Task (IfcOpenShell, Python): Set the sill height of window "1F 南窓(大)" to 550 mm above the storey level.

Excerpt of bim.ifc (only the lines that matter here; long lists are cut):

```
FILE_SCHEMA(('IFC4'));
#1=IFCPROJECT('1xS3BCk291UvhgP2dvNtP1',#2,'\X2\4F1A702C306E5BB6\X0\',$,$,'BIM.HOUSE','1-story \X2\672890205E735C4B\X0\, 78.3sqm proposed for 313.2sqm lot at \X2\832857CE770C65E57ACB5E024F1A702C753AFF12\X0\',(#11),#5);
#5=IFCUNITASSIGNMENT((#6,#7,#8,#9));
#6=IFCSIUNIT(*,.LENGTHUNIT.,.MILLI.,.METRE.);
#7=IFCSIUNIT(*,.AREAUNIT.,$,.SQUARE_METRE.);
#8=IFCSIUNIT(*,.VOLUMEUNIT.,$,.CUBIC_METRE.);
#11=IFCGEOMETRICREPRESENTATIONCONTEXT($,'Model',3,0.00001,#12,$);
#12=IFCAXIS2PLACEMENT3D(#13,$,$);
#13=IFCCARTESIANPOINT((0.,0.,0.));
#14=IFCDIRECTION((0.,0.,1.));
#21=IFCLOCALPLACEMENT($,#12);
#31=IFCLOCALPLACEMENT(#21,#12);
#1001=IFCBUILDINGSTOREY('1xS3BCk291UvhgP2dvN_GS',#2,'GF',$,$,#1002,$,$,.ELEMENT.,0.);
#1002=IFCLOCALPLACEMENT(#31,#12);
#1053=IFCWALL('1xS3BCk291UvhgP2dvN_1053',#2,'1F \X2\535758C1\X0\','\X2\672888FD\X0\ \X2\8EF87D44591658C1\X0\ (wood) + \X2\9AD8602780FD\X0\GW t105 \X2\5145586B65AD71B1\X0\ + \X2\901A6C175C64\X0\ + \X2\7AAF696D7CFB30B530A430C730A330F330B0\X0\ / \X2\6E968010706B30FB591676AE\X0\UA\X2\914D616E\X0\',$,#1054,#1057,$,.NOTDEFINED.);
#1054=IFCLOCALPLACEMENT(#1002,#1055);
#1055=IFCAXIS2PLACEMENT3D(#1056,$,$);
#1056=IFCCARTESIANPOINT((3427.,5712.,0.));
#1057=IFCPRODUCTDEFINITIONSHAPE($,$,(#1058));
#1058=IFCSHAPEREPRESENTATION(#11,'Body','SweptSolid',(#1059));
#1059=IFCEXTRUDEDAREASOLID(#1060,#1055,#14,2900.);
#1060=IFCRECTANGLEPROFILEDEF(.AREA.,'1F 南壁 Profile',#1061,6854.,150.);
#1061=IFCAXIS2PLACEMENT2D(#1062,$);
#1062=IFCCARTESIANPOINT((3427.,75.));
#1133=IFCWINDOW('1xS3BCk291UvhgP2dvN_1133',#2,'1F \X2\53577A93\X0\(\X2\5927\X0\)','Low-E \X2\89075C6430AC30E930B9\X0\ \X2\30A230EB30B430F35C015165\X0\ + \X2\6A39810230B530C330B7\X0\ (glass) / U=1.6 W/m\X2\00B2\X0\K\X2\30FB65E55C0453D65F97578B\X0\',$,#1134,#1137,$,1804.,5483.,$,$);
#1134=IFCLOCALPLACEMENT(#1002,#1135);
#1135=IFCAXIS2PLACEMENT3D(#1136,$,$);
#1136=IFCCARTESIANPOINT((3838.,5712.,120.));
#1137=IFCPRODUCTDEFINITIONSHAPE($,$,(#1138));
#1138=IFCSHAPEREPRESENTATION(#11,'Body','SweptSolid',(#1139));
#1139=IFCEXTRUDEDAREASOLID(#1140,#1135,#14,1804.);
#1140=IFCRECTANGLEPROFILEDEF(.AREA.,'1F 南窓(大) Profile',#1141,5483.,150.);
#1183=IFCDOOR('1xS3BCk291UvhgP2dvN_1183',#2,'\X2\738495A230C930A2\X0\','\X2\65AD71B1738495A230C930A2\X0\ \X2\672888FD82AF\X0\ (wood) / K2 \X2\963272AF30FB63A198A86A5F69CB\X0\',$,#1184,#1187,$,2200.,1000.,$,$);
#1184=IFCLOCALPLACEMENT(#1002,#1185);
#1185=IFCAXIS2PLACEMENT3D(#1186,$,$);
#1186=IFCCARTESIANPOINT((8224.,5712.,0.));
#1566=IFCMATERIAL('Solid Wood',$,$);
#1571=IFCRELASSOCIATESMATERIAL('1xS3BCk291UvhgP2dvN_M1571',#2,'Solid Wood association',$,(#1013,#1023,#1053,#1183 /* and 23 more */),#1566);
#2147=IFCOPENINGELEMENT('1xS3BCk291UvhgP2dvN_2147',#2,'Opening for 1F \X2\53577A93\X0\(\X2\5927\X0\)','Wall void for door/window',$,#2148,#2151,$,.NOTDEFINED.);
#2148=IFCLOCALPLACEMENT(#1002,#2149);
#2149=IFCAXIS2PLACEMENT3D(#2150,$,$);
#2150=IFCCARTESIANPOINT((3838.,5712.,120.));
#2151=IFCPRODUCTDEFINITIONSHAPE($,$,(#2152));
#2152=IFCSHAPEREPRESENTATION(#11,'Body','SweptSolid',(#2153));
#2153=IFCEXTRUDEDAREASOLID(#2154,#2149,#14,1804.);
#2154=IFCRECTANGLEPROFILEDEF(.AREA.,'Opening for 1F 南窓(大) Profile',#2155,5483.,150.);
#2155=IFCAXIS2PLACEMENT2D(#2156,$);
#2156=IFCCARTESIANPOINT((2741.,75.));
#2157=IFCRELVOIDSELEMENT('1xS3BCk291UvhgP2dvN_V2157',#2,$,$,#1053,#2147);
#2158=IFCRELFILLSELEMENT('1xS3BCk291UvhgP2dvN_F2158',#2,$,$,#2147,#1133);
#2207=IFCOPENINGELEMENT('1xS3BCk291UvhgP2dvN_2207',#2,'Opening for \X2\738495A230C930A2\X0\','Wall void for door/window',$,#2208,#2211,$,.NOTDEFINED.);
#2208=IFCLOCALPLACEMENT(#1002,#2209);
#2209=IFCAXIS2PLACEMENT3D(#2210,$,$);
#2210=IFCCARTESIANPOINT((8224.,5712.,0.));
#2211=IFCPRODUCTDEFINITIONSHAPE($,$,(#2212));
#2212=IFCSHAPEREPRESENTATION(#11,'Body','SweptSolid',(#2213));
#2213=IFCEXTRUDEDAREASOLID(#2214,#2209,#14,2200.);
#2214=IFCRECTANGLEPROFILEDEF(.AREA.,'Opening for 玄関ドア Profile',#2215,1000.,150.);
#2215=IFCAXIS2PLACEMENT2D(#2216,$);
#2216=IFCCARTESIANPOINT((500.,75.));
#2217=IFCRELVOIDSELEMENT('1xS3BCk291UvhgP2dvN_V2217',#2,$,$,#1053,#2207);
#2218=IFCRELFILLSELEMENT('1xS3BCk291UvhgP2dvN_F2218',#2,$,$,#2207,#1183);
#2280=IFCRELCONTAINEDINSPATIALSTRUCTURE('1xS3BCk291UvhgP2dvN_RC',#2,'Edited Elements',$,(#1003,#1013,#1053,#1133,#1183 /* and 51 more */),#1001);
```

```python
import numpy as np
import ifcopenshell
import ifcopenshell.api.geometry
import ifcopenshell.geom
import ifcopenshell.util.element
import ifcopenshell.util.placement
import ifcopenshell.util.shape
import ifcopenshell.util.unit

model = ifcopenshell.open("bim.ifc")
unit_scale = ifcopenshell.util.unit.calculate_unit_scale(model)

window = model.by_guid("1xS3BCk291UvhgP2dvN_1133")
opening = window.FillsVoids[0].RelatingOpeningElement
storey = ifcopenshell.util.element.get_container(window, ifc_class="IfcBuildingStorey")
level = ifcopenshell.util.placement.get_local_placement(storey.ObjectPlacement)[2, 3]

# The opening's origin need not be at the sill, so measure its lowest point.
shape = ifcopenshell.geom.create_shape(ifcopenshell.geom.settings(), opening)
bottom = ifcopenshell.util.shape.get_shape_bottom_elevation(shape, shape.geometry) / unit_scale
dz = level + 550.0 - bottom

shift = np.array([0.0, 0.0, dz])
# The window is not placed relative to its opening, so move both.
for product in (opening, window):
    matrix = ifcopenshell.util.placement.get_local_placement(product.ObjectPlacement)
    matrix[:3, 3] += shift
    ifcopenshell.api.geometry.edit_object_placement(model, product=product, matrix=matrix, is_si=False)

print(f"moved by {dz * unit_scale:+.3f} m")

model.write("bim_rev.ifc")
```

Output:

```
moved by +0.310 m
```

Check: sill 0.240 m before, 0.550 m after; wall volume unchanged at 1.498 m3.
